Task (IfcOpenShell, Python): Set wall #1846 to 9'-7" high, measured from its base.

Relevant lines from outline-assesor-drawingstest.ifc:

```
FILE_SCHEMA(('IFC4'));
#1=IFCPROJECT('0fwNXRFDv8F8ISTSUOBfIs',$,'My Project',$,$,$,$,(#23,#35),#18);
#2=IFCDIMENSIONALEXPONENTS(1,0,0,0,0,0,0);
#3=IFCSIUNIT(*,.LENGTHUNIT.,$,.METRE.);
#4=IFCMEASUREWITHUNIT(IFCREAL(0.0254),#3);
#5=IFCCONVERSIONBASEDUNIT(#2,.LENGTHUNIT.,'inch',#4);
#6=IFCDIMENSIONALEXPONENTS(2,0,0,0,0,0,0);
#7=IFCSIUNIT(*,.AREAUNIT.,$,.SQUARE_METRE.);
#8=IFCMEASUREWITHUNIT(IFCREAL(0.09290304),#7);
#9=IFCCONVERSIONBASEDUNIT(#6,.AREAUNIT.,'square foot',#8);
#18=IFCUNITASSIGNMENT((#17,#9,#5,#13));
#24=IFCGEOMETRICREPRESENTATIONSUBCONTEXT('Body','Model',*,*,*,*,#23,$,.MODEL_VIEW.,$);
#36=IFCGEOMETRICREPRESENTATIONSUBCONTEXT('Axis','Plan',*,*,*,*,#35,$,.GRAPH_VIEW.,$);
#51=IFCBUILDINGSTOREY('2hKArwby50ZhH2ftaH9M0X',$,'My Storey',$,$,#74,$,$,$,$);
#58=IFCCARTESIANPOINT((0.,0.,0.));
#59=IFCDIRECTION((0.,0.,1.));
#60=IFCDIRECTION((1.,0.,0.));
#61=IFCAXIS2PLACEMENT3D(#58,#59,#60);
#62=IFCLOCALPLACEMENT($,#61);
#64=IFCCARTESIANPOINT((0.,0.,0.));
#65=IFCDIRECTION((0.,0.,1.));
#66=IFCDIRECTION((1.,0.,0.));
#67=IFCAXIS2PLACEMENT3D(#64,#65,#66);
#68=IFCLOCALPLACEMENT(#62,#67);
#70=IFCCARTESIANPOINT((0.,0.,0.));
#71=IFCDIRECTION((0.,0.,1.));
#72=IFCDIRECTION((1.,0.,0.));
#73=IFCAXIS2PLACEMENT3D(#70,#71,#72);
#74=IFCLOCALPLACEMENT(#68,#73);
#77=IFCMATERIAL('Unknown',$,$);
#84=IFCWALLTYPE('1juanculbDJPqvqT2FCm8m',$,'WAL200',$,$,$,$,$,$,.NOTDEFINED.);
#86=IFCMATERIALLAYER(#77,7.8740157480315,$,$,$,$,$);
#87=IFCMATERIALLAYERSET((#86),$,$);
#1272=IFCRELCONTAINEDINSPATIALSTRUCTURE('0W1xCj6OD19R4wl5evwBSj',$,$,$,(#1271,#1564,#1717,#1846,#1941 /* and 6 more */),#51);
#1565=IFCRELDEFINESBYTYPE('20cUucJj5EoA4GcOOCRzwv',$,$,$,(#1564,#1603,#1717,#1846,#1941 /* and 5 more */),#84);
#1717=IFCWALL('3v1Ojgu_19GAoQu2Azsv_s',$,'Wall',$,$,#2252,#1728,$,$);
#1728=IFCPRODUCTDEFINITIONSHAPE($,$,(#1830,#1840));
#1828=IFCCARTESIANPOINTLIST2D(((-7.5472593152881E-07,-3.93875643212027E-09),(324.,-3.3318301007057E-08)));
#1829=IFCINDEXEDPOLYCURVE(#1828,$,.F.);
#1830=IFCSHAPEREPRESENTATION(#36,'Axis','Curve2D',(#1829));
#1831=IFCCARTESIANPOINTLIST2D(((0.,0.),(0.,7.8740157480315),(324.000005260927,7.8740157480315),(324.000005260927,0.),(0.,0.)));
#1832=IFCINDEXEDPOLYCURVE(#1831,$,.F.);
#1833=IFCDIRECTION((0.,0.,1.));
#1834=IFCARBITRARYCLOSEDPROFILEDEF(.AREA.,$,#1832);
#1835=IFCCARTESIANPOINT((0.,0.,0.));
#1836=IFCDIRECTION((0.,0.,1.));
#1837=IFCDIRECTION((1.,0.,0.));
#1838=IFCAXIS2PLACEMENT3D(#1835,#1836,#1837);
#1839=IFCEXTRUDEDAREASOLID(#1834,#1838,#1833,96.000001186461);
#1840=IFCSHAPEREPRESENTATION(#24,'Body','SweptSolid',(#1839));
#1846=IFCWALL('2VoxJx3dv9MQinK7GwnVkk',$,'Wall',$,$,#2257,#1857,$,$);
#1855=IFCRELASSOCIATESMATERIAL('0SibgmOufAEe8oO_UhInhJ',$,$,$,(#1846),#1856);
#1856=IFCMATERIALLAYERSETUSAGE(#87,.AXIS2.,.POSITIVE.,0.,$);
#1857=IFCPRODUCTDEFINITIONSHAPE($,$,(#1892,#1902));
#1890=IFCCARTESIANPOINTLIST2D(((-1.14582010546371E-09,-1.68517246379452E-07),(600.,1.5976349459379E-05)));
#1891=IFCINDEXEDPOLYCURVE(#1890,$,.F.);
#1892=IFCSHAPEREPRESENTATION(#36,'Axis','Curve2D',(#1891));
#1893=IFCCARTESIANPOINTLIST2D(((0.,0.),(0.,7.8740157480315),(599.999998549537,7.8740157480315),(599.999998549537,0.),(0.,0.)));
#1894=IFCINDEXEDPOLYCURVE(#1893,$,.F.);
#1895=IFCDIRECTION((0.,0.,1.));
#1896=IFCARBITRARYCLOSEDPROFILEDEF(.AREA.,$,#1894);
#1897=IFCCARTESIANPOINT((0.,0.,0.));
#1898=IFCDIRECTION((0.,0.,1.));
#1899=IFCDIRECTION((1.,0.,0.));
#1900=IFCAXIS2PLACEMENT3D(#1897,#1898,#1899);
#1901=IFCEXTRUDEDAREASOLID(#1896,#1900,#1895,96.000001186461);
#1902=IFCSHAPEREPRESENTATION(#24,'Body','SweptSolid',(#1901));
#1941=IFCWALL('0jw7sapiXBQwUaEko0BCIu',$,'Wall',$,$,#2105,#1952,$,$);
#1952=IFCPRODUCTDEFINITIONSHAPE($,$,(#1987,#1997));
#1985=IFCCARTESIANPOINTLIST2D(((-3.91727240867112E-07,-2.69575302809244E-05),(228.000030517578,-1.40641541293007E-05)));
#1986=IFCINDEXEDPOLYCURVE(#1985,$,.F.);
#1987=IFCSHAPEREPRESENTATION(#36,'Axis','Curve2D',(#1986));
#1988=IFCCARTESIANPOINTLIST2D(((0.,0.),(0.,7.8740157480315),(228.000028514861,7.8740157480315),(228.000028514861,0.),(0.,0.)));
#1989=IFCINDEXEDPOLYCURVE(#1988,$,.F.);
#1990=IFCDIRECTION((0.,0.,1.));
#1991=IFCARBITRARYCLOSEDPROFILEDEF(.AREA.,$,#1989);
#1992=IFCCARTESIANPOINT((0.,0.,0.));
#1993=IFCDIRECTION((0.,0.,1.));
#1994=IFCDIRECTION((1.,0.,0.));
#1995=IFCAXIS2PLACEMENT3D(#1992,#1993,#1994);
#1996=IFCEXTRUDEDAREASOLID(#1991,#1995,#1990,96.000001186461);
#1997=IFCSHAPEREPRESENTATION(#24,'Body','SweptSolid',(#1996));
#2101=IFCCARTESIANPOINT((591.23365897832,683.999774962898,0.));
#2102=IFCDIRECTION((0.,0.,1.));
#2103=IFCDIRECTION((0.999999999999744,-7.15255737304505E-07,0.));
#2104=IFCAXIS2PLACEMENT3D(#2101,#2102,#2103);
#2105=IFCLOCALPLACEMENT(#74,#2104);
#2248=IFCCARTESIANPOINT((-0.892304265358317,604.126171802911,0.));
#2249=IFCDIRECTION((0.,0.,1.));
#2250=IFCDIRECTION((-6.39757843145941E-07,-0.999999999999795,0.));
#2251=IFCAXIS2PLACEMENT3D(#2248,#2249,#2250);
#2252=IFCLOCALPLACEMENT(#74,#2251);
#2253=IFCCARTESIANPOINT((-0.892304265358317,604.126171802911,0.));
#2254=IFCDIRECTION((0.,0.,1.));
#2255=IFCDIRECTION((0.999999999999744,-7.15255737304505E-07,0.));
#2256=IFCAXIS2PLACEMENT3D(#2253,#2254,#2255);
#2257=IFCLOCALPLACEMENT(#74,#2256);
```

```python
import ifcopenshell
import ifcopenshell.geom
import ifcopenshell.util.representation
import ifcopenshell.util.shape
import ifcopenshell.util.unit

model = ifcopenshell.open("outline-assesor-drawingstest.ifc")
unit_scale = ifcopenshell.util.unit.calculate_unit_scale(model)
settings = ifcopenshell.geom.settings()


def volume(element):
    """Net volume in cubic metres, openings subtracted."""
    shape = ifcopenshell.geom.create_shape(settings, element)
    return ifcopenshell.util.shape.get_volume(shape.geometry)


wall = model.by_guid("2VoxJx3dv9MQinK7GwnVkk")
before = volume(wall)

body = ifcopenshell.util.representation.get_representation(wall, "Model", "Body")
solid = body.Items[0]
old_height = solid.Depth
solid.Depth = 115 * 0.0254 / unit_scale
after = volume(wall)

print(f"height {old_height:g} -> {solid.Depth:g}, volume {before:.3f} -> {after:.3f} m3")

model.write("outline-assesor-drawingstest_updated.ifc")
```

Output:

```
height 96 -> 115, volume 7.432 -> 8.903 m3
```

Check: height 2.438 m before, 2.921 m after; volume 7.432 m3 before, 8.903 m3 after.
